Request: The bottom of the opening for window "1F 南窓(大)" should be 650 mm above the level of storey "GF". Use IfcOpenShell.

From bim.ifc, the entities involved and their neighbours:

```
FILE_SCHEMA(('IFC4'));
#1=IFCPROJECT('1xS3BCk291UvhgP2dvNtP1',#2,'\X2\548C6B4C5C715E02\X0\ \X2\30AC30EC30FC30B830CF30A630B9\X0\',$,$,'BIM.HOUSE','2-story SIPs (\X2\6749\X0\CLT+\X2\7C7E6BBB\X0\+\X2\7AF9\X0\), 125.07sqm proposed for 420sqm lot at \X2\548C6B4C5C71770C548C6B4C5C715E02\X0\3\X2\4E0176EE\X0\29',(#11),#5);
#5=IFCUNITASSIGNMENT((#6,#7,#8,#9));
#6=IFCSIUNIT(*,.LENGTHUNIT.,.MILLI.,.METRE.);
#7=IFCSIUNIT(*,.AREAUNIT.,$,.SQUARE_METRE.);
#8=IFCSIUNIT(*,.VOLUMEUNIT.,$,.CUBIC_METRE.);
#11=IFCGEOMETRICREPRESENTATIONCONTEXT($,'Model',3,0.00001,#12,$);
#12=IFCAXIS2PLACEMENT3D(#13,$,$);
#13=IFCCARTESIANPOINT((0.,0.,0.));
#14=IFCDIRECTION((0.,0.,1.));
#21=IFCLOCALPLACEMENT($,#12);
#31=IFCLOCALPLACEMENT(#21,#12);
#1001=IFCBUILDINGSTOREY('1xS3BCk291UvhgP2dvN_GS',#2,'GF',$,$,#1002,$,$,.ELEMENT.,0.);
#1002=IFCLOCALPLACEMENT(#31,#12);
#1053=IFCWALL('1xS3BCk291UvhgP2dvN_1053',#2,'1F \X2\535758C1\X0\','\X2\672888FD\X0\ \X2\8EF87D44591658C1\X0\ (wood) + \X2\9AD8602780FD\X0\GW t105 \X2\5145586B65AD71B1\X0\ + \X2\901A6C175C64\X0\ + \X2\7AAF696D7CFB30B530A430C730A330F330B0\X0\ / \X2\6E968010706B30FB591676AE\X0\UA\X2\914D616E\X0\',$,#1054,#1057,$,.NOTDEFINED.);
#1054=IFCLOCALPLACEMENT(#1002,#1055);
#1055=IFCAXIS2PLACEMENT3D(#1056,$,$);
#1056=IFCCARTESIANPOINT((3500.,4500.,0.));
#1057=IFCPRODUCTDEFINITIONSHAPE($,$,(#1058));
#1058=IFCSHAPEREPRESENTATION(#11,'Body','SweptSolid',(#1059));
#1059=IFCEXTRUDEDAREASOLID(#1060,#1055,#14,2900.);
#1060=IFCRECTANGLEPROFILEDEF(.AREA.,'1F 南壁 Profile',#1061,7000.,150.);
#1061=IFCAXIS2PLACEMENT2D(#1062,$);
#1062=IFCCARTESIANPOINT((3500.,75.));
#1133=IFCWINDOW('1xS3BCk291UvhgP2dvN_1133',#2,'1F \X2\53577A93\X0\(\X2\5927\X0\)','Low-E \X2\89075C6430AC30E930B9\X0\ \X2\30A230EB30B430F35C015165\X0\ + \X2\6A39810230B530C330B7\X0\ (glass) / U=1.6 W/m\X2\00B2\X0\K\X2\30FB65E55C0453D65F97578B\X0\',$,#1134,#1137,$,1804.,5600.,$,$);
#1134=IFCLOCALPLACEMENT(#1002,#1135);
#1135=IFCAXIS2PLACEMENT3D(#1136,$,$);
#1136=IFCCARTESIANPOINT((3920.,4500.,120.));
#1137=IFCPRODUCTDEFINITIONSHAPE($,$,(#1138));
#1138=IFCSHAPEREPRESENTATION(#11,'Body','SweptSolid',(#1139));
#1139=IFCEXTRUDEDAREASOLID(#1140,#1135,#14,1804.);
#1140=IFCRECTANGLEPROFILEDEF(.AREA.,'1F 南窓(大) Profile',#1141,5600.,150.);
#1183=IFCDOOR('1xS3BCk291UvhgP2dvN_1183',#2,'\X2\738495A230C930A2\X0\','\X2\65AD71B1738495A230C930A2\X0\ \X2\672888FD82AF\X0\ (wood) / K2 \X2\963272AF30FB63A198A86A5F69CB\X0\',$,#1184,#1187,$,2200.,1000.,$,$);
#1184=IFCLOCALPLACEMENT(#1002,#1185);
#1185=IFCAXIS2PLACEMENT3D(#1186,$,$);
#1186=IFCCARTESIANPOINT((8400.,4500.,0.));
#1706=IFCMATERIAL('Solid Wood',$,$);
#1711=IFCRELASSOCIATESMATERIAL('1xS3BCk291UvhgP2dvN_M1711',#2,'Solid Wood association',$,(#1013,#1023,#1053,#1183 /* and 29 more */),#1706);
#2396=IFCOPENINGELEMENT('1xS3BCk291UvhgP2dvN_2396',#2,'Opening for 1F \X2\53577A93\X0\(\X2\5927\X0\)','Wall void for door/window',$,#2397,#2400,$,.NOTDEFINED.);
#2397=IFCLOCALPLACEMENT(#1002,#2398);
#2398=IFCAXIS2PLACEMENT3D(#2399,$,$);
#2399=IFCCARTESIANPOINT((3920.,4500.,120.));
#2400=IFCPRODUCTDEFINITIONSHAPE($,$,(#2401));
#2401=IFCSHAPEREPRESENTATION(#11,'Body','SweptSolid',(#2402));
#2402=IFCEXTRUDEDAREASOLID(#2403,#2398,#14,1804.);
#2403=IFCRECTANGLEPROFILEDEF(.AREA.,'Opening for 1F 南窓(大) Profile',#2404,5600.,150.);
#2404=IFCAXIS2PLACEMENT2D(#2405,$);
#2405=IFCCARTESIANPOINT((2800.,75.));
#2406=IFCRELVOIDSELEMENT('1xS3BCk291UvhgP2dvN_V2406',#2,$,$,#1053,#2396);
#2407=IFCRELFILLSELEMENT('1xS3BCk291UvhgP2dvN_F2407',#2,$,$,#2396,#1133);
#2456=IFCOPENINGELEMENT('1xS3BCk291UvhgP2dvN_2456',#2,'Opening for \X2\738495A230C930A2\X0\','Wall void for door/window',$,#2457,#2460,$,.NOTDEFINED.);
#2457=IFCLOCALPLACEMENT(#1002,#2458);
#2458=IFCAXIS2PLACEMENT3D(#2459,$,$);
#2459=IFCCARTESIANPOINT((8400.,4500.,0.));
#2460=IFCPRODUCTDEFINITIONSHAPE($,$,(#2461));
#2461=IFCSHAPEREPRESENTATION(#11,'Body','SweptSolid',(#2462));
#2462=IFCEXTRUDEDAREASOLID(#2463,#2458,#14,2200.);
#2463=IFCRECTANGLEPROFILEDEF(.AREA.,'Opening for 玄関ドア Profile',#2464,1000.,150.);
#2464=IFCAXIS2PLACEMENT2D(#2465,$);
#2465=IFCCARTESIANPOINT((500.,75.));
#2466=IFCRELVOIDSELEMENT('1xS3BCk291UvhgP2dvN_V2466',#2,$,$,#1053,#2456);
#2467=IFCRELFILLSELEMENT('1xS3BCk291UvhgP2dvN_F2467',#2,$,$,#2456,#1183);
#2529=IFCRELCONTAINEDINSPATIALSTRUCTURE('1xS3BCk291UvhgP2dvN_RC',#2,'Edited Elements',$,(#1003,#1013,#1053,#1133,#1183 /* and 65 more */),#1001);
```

```python
import numpy as np
import ifcopenshell
import ifcopenshell.api.geometry
import ifcopenshell.geom
import ifcopenshell.util.element
import ifcopenshell.util.placement
import ifcopenshell.util.shape
import ifcopenshell.util.unit

model = ifcopenshell.open("bim.ifc")
unit_scale = ifcopenshell.util.unit.calculate_unit_scale(model)

window = model.by_guid("1xS3BCk291UvhgP2dvN_1133")
opening = window.FillsVoids[0].RelatingOpeningElement
storey = ifcopenshell.util.element.get_container(window, ifc_class="IfcBuildingStorey")
level = ifcopenshell.util.placement.get_local_placement(storey.ObjectPlacement)[2, 3]

# The opening's origin need not be at the sill, so measure its lowest point.
shape = ifcopenshell.geom.create_shape(ifcopenshell.geom.settings(), opening)
bottom = ifcopenshell.util.shape.get_shape_bottom_elevation(shape, shape.geometry) / unit_scale
dz = level + 0.65 / unit_scale - bottom

shift = np.array([0.0, 0.0, dz])
# The window is not placed relative to its opening, so move both.
for product in (opening, window):
    matrix = ifcopenshell.util.placement.get_local_placement(product.ObjectPlacement)
    matrix[:3, 3] += shift
    ifcopenshell.api.geometry.edit_object_placement(model, product=product, matrix=matrix, is_si=False)

print(f"moved by {dz * unit_scale:+.3f} m")

model.write("bim_rev.ifc")
```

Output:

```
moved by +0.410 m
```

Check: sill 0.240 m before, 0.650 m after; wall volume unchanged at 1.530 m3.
